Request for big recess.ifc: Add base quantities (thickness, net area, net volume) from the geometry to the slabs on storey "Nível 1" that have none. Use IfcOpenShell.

First a look at what the model holds.

```python
import ifcopenshell
import ifcopenshell.util.element
import ifcopenshell.util.unit

model = ifcopenshell.open("big recess.ifc")
print(model.schema)
for unit_type in ("LENGTHUNIT", "AREAUNIT", "VOLUMEUNIT"):
    print(unit_type, ifcopenshell.util.unit.calculate_unit_scale(model, unit_type))
storey = next(s for s in model.by_type("IfcBuildingStorey") if s.Name == "Nível 1")
slabs = [e for e in ifcopenshell.util.element.get_decomposition(storey) if e.is_a("IfcSlab")]
for e in sorted(slabs, key=lambda e: e.id()):
    print(e.id(), e.is_a(), e.Name, list(ifcopenshell.util.element.get_psets(e, qtos_only=True)), sep=" | ")
```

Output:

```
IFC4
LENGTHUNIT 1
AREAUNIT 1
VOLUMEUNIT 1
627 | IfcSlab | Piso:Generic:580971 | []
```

```python
import ifcopenshell
import ifcopenshell.api.pset
import ifcopenshell.geom
import ifcopenshell.util.element
import ifcopenshell.util.shape
import ifcopenshell.util.unit

model = ifcopenshell.open("big recess.ifc")
unit_scale = ifcopenshell.util.unit.calculate_unit_scale(model)
area_scale = ifcopenshell.util.unit.calculate_unit_scale(model, "AREAUNIT")
volume_scale = ifcopenshell.util.unit.calculate_unit_scale(model, "VOLUMEUNIT")
settings = ifcopenshell.geom.settings()

storey = next(s for s in model.by_type("IfcBuildingStorey") if s.Name == "Nível 1")
slabs = [e for e in ifcopenshell.util.element.get_decomposition(storey) if e.is_a("IfcSlab")]

for e in sorted(slabs, key=lambda e: e.id()):
    if ifcopenshell.util.element.get_psets(e, qtos_only=True, should_inherit=False):
        continue
    # Geometry comes back in metres, in the element's own axes.
    shape = ifcopenshell.geom.create_shape(settings, e)
    values = {
        "Width": ifcopenshell.util.shape.get_z(shape.geometry) / unit_scale,
        "NetArea": ifcopenshell.util.shape.get_footprint_area(shape.geometry) / area_scale,
        "NetVolume": ifcopenshell.util.shape.get_volume(shape.geometry) / volume_scale,
    }
    qto = ifcopenshell.api.pset.add_qto(model, product=e, name="Qto_SlabBaseQuantities")
    ifcopenshell.api.pset.edit_qto(model, qto=qto, properties=values)
    print(e.id(), {k: round(v, 3) for k, v in values.items()})

model.write("big recess_updated.ifc")
```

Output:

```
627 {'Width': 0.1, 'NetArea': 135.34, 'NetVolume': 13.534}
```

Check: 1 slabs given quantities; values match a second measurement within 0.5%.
